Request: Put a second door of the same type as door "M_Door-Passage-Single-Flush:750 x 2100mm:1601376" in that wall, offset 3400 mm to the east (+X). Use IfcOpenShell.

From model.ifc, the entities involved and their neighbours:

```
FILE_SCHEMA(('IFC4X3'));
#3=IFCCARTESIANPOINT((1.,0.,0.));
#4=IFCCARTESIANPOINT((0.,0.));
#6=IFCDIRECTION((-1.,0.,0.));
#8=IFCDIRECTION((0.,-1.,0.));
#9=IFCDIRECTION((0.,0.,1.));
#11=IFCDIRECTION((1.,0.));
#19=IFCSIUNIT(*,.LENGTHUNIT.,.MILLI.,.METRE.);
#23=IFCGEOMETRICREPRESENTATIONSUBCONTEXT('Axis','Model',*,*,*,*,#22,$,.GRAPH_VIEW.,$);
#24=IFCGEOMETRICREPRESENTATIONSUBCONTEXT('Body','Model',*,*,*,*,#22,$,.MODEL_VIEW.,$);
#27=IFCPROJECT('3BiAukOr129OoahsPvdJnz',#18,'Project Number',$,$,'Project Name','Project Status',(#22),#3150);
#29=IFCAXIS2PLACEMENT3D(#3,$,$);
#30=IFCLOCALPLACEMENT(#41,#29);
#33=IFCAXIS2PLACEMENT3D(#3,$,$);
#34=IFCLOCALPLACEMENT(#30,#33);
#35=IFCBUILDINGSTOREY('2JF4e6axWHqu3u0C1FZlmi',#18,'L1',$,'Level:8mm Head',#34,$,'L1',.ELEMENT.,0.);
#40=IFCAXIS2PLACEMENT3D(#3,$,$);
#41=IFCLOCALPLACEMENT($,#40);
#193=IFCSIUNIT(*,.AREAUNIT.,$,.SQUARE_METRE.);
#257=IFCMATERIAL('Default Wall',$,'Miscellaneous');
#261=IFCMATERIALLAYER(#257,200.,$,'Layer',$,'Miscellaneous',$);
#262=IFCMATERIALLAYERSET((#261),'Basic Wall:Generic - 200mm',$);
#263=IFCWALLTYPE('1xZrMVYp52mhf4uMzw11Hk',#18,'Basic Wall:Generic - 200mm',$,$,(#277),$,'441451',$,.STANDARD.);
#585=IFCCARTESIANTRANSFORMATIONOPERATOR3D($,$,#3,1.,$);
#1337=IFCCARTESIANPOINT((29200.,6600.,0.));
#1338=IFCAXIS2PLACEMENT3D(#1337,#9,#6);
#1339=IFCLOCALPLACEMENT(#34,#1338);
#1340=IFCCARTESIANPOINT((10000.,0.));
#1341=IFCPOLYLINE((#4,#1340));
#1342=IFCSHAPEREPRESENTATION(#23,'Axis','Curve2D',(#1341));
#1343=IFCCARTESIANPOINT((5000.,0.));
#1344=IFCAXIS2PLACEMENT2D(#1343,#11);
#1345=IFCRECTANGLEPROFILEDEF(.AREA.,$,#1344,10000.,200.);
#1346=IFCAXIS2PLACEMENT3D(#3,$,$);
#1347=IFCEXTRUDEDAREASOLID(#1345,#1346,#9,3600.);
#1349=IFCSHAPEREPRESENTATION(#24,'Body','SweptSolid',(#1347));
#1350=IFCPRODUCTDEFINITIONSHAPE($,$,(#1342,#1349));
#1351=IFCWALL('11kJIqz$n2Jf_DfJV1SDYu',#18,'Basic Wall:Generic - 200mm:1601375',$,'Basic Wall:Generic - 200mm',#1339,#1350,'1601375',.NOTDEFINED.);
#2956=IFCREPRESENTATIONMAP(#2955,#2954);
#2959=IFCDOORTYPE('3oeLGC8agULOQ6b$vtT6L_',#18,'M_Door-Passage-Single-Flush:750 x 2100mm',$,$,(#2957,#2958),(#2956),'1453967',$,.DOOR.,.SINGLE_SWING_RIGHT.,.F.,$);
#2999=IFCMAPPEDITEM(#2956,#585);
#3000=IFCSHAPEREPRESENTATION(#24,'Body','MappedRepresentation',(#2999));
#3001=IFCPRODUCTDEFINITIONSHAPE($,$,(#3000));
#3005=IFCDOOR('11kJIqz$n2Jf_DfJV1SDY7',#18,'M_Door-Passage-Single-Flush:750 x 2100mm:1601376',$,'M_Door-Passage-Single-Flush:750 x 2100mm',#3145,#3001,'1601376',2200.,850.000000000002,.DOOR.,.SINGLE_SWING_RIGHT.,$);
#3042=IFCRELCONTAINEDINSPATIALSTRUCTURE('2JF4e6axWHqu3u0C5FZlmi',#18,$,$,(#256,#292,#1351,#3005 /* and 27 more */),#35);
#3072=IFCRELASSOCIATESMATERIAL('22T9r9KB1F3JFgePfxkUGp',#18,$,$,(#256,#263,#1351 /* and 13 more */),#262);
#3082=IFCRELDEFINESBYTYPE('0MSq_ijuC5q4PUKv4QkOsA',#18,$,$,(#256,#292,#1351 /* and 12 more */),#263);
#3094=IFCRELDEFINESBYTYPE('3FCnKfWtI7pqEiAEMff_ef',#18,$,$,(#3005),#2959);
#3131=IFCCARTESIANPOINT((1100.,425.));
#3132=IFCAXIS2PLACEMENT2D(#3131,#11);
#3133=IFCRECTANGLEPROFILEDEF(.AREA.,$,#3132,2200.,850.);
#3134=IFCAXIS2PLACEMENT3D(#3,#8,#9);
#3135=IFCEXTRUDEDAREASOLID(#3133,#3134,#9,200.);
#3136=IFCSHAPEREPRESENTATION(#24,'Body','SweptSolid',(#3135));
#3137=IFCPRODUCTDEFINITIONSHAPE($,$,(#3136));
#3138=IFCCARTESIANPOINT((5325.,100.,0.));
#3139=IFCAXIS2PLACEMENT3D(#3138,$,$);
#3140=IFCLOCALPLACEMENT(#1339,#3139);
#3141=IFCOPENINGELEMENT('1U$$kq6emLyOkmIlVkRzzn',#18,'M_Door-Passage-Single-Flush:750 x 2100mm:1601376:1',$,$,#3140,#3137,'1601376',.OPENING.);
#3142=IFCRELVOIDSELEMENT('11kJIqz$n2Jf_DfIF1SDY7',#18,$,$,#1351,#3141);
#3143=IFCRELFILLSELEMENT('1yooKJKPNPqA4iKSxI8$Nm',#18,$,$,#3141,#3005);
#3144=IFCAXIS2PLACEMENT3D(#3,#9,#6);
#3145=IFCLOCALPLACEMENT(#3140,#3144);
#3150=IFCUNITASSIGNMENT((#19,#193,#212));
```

```python
import ifcopenshell
import ifcopenshell.api.feature
import ifcopenshell.api.geometry
import ifcopenshell.api.root
import ifcopenshell.geom
import ifcopenshell.util.element
import ifcopenshell.util.placement
import ifcopenshell.util.shape

model = ifcopenshell.open("model.ifc")
settings = ifcopenshell.geom.settings()


def volume(element):
    """Net volume in cubic metres, openings subtracted."""
    shape = ifcopenshell.geom.create_shape(settings, element)
    return ifcopenshell.util.shape.get_volume(shape.geometry)


def reuse_history(source, copy):
    """copy_class also copies each property set's owner history, people and application; keep the originals."""
    for rel in copy.IsDefinedBy:
        if rel.is_a("IfcRelDefinesByProperties") and (history := rel.RelatingPropertyDefinition.OwnerHistory):
            rel.RelatingPropertyDefinition.OwnerHistory = source.OwnerHistory
            ifcopenshell.util.element.remove_deep2(model, history)


door = model.by_guid("11kJIqz$n2Jf_DfJV1SDY7")
opening = door.FillsVoids[0].RelatingOpeningElement
wall = opening.VoidsElements[0].RelatingBuildingElement
before = volume(wall)
shift = ifcopenshell.util.placement.get_local_placement(wall.ObjectPlacement)[:3, 0] * -3400.0

# copy_class copies the void relationship, type, container and properties, but no geometry.
new_opening = ifcopenshell.api.root.copy_class(model, product=opening)
new_opening.Representation = ifcopenshell.util.element.copy_deep(
    model, opening.Representation, exclude=["IfcGeometricRepresentationContext", "IfcRepresentationMap"]
)
new_opening.Name = "M_Door-Passage-Single-Flush:750 x 2100mm"
new_opening.Tag = None
new_door = ifcopenshell.api.root.copy_class(model, product=door)
new_door.Representation = ifcopenshell.util.element.copy_deep(
    model, door.Representation, exclude=["IfcGeometricRepresentationContext", "IfcRepresentationMap"]
)
new_door.Name = "M_Door-Passage-Single-Flush:750 x 2100mm"
new_door.Tag = None
reuse_history(door, new_door)
ifcopenshell.api.feature.add_filling(model, opening=new_opening, element=new_door)

for old, new in ((opening, new_opening), (door, new_door)):
    matrix = ifcopenshell.util.placement.get_local_placement(old.ObjectPlacement)
    matrix[:3, 3] += shift
    ifcopenshell.api.geometry.edit_object_placement(model, product=new, matrix=matrix, is_si=False)

after = volume(wall)

print(f"wall volume {before:.3f} -> {after:.3f} m3")

model.write("model_updated.ifc")
```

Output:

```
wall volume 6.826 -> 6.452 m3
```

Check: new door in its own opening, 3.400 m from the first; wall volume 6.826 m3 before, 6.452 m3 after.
